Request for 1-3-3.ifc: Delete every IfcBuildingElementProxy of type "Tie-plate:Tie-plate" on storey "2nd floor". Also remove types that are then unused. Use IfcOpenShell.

First a look at what the model holds.

```python
import ifcopenshell
import ifcopenshell.util.element

model = ifcopenshell.open("1-3-3.ifc")
print(model.schema)
storey = next(s for s in model.by_type("IfcBuildingStorey") if s.Name == "2nd floor")
proxies = [e for e in ifcopenshell.util.element.get_decomposition(storey) if e.is_a("IfcBuildingElementProxy")]
seen = {}
for e in proxies:
    element_type = ifcopenshell.util.element.get_type(e)
    name = element_type.Name if element_type not in (None, e) else None
    seen[name] = seen.get(name, 0) + 1
for name, count in sorted(seen.items(), key=str):
    print(count, "x", name)
```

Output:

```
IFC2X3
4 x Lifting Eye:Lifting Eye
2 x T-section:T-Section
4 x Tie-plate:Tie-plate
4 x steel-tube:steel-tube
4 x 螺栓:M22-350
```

```python
import ifcopenshell
import ifcopenshell.api.root
import ifcopenshell.util.element

model = ifcopenshell.open("1-3-3.ifc")

storey = next(s for s in model.by_type("IfcBuildingStorey") if s.Name == "2nd floor")
proxies = [e for e in ifcopenshell.util.element.get_decomposition(storey) if e.is_a("IfcBuildingElementProxy")]
targets = [e for e in proxies if (t := ifcopenshell.util.element.get_type(e)) not in (None, e) and t.Name == "Tie-plate:Tie-plate"]
types = {ifcopenshell.util.element.get_type(e) for e in targets} - {None, *targets}

for e in targets:
    ifcopenshell.api.root.remove_product(model, product=e)
print(len(targets), "removed")

unused = [t for t in types if not ifcopenshell.util.element.get_types(t)]
for t in unused:
    ifcopenshell.api.root.remove_product(model, product=t)
print(len(unused), "unused types removed")

model.write("1-3-3_rev.ifc")
```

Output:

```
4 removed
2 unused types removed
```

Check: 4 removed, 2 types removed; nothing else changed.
